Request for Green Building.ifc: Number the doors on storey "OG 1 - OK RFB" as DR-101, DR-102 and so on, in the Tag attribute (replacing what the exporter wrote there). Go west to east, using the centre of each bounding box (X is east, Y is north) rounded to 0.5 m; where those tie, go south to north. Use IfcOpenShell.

First a look at what the model holds.

```python
import ifcopenshell
import ifcopenshell.util.element
import ifcopenshell.util.placement

model = ifcopenshell.open("Green Building.ifc")
print(model.schema)
storey = next(s for s in model.by_type("IfcBuildingStorey") if s.Name == "OG 1 - OK RFB")
doors = [e for e in ifcopenshell.util.element.get_decomposition(storey) if e.is_a("IfcDoor")]
for e in sorted(doors, key=lambda e: e.id()):
    origin = ifcopenshell.util.placement.get_local_placement(e.ObjectPlacement)[:3, 3]
    print(e.id(), e.Tag, e.Name, origin.round(2) + 0.0, sep=" | ")
```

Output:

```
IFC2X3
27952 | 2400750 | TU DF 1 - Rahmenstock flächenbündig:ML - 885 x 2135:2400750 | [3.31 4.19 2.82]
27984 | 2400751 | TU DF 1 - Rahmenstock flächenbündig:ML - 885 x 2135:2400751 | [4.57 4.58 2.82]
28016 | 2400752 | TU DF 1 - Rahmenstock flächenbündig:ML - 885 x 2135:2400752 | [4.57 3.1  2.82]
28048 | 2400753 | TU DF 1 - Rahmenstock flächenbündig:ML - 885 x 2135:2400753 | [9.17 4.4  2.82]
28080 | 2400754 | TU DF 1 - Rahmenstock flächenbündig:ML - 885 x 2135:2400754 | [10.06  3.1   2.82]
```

```python
import ifcopenshell
import ifcopenshell.geom
import ifcopenshell.util.element
import ifcopenshell.util.shape

model = ifcopenshell.open("Green Building.ifc")
settings = ifcopenshell.geom.settings()
settings.set("use-world-coords", True)


def centre(element):
    shape = ifcopenshell.geom.create_shape(settings, element)
    return ifcopenshell.util.shape.get_bbox_centroid(shape.geometry)


storey = next(s for s in model.by_type("IfcBuildingStorey") if s.Name == "OG 1 - OK RFB")
doors = [e for e in ifcopenshell.util.element.get_decomposition(storey) if e.is_a("IfcDoor")]

# Insertion points can sit at a corner or the storey origin, so sort by the geometry (in metres).
centres = {e: centre(e) for e in doors}
doors.sort(key=lambda e: (round(centres[e][0] / 0.5), centres[e][1]))

for i, e in enumerate(doors, start=1):
    number = f"DR-1{i:02d}"
    e.Tag = number
    print(e.id(), number)

model.write("Green Building_v2.ifc")
```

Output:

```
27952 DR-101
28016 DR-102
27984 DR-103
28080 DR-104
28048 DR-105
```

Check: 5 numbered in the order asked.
